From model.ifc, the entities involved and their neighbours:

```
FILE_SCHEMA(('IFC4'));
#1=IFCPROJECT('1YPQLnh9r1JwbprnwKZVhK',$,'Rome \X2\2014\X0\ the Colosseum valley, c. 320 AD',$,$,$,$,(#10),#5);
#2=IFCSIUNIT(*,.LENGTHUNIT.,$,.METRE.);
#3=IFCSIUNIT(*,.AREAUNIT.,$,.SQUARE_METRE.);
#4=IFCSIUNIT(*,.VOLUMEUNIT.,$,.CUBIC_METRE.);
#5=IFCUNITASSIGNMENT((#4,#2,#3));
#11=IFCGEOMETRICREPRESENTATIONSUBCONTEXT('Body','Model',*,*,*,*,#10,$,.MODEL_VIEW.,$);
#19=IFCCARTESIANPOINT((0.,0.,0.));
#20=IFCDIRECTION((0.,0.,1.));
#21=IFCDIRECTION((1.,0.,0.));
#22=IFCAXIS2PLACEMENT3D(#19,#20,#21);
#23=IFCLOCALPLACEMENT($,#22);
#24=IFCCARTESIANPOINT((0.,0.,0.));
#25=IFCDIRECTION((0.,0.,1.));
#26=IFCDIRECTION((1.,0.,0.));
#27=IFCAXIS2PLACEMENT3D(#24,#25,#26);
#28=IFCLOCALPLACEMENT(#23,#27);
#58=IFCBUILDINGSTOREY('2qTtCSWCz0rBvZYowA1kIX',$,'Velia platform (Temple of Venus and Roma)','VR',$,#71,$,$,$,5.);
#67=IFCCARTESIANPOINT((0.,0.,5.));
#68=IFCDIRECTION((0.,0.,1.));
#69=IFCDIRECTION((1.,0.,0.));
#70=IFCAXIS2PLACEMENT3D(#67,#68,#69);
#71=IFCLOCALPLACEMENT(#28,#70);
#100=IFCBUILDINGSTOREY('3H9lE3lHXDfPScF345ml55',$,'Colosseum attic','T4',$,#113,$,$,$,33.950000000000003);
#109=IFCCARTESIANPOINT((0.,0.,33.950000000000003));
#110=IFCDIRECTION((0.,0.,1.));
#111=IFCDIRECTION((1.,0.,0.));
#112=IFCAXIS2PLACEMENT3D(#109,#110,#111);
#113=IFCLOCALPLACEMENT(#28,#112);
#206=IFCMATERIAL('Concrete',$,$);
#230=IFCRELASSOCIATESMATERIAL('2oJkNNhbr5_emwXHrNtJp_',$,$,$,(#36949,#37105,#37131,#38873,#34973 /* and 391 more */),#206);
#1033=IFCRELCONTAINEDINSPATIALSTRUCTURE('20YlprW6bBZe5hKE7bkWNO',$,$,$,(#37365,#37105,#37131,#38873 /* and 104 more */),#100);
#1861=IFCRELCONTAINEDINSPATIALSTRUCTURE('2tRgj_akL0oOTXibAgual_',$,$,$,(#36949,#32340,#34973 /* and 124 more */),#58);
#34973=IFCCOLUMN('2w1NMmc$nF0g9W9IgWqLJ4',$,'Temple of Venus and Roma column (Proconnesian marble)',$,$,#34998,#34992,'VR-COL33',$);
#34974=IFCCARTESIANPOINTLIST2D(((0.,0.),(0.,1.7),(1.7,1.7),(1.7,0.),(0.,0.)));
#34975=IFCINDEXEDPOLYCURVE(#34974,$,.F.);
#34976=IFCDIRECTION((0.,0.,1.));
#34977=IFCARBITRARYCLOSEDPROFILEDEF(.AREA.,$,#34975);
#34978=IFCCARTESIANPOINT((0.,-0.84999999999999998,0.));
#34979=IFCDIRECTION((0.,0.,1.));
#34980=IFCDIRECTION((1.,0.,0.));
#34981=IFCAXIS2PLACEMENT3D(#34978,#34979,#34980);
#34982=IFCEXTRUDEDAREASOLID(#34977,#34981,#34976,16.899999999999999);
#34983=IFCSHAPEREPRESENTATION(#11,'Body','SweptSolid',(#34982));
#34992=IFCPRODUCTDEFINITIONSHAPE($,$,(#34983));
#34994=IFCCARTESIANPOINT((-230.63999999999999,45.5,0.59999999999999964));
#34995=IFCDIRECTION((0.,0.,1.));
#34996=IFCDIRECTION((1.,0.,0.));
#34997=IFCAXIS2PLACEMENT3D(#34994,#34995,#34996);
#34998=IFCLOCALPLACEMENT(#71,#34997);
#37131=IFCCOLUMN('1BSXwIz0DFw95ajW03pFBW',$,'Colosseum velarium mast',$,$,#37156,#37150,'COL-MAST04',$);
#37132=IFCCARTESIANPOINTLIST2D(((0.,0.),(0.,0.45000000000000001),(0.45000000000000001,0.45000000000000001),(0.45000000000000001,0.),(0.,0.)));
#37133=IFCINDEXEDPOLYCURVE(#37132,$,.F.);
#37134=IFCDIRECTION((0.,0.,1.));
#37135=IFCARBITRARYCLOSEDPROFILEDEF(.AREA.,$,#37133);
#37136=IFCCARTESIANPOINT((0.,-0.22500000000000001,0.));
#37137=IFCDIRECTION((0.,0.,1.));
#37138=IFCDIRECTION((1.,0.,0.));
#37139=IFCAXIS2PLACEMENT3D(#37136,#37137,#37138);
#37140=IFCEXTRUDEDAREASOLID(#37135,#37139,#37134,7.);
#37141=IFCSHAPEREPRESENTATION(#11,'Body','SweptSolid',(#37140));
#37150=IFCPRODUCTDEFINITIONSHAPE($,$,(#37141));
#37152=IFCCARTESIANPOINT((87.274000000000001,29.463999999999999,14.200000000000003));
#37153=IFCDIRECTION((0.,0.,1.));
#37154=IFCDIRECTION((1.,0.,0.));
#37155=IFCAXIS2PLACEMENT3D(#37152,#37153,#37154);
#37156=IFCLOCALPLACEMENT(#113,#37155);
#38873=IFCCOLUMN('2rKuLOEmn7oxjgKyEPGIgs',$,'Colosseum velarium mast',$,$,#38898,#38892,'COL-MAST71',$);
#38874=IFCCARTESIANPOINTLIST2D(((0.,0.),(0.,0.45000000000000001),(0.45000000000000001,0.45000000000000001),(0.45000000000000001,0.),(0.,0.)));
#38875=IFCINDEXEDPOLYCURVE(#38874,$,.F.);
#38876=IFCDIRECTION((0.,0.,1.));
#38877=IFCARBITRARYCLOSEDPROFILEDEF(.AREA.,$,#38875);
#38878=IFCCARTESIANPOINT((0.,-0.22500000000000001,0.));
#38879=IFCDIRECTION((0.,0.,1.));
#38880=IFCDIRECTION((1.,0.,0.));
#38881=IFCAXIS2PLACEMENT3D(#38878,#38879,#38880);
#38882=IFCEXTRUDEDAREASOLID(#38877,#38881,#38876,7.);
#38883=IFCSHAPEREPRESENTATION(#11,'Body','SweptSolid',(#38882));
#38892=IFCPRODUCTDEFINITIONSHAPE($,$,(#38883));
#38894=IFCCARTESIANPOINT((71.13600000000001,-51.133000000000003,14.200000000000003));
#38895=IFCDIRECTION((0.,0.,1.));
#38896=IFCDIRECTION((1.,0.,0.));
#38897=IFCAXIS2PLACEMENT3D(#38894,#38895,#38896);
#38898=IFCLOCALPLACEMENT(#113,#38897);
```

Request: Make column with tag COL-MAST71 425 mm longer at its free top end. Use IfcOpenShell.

```python
import ifcopenshell
import ifcopenshell.util.representation
import ifcopenshell.util.unit

model = ifcopenshell.open("model.ifc")
unit_scale = ifcopenshell.util.unit.calculate_unit_scale(model)

member = model.by_guid("2rKuLOEmn7oxjgKyEPGIgs")
change = 0.425 / unit_scale

# The extrusion runs towards the end named, so only its depth changes.
body = ifcopenshell.util.representation.get_representation(member, "Model", "Body")
solid = body.Items[0]
old_length = solid.Depth
solid.Depth += change

print(f"length {old_length:g} -> {solid.Depth:g}")

model.write("model_rev.ifc")
```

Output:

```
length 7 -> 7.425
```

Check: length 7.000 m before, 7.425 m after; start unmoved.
